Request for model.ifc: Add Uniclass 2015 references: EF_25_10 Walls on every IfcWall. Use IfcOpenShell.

First a look at what the model holds.

```python
import ifcopenshell

model = ifcopenshell.open("model.ifc")
print(model.schema)
print("classifications:", [c.Name for c in model.by_type("IfcClassification")])
for ifc_class in ("IfcDoor", "IfcRoof", "IfcStair", "IfcWall", "IfcWindow"):
    print(ifc_class, len(model.by_type(ifc_class)))
```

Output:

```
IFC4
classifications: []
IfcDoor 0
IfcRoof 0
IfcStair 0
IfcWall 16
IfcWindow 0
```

```python
import ifcopenshell
import ifcopenshell.api.classification

model = ifcopenshell.open("model.ifc")

system = ifcopenshell.api.classification.add_classification(model, classification="Uniclass 2015")

codes = {
    "IfcWall": ("EF_25_10", "Walls"),
}
for ifc_class, (code, name) in codes.items():
    products = model.by_type(ifc_class)
    ifcopenshell.api.classification.add_reference(
        model, products=products, classification=system, identification=code, name=name
    )
    print(code, len(products))

model.write("model_updated.ifc")
```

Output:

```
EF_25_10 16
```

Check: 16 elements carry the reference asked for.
